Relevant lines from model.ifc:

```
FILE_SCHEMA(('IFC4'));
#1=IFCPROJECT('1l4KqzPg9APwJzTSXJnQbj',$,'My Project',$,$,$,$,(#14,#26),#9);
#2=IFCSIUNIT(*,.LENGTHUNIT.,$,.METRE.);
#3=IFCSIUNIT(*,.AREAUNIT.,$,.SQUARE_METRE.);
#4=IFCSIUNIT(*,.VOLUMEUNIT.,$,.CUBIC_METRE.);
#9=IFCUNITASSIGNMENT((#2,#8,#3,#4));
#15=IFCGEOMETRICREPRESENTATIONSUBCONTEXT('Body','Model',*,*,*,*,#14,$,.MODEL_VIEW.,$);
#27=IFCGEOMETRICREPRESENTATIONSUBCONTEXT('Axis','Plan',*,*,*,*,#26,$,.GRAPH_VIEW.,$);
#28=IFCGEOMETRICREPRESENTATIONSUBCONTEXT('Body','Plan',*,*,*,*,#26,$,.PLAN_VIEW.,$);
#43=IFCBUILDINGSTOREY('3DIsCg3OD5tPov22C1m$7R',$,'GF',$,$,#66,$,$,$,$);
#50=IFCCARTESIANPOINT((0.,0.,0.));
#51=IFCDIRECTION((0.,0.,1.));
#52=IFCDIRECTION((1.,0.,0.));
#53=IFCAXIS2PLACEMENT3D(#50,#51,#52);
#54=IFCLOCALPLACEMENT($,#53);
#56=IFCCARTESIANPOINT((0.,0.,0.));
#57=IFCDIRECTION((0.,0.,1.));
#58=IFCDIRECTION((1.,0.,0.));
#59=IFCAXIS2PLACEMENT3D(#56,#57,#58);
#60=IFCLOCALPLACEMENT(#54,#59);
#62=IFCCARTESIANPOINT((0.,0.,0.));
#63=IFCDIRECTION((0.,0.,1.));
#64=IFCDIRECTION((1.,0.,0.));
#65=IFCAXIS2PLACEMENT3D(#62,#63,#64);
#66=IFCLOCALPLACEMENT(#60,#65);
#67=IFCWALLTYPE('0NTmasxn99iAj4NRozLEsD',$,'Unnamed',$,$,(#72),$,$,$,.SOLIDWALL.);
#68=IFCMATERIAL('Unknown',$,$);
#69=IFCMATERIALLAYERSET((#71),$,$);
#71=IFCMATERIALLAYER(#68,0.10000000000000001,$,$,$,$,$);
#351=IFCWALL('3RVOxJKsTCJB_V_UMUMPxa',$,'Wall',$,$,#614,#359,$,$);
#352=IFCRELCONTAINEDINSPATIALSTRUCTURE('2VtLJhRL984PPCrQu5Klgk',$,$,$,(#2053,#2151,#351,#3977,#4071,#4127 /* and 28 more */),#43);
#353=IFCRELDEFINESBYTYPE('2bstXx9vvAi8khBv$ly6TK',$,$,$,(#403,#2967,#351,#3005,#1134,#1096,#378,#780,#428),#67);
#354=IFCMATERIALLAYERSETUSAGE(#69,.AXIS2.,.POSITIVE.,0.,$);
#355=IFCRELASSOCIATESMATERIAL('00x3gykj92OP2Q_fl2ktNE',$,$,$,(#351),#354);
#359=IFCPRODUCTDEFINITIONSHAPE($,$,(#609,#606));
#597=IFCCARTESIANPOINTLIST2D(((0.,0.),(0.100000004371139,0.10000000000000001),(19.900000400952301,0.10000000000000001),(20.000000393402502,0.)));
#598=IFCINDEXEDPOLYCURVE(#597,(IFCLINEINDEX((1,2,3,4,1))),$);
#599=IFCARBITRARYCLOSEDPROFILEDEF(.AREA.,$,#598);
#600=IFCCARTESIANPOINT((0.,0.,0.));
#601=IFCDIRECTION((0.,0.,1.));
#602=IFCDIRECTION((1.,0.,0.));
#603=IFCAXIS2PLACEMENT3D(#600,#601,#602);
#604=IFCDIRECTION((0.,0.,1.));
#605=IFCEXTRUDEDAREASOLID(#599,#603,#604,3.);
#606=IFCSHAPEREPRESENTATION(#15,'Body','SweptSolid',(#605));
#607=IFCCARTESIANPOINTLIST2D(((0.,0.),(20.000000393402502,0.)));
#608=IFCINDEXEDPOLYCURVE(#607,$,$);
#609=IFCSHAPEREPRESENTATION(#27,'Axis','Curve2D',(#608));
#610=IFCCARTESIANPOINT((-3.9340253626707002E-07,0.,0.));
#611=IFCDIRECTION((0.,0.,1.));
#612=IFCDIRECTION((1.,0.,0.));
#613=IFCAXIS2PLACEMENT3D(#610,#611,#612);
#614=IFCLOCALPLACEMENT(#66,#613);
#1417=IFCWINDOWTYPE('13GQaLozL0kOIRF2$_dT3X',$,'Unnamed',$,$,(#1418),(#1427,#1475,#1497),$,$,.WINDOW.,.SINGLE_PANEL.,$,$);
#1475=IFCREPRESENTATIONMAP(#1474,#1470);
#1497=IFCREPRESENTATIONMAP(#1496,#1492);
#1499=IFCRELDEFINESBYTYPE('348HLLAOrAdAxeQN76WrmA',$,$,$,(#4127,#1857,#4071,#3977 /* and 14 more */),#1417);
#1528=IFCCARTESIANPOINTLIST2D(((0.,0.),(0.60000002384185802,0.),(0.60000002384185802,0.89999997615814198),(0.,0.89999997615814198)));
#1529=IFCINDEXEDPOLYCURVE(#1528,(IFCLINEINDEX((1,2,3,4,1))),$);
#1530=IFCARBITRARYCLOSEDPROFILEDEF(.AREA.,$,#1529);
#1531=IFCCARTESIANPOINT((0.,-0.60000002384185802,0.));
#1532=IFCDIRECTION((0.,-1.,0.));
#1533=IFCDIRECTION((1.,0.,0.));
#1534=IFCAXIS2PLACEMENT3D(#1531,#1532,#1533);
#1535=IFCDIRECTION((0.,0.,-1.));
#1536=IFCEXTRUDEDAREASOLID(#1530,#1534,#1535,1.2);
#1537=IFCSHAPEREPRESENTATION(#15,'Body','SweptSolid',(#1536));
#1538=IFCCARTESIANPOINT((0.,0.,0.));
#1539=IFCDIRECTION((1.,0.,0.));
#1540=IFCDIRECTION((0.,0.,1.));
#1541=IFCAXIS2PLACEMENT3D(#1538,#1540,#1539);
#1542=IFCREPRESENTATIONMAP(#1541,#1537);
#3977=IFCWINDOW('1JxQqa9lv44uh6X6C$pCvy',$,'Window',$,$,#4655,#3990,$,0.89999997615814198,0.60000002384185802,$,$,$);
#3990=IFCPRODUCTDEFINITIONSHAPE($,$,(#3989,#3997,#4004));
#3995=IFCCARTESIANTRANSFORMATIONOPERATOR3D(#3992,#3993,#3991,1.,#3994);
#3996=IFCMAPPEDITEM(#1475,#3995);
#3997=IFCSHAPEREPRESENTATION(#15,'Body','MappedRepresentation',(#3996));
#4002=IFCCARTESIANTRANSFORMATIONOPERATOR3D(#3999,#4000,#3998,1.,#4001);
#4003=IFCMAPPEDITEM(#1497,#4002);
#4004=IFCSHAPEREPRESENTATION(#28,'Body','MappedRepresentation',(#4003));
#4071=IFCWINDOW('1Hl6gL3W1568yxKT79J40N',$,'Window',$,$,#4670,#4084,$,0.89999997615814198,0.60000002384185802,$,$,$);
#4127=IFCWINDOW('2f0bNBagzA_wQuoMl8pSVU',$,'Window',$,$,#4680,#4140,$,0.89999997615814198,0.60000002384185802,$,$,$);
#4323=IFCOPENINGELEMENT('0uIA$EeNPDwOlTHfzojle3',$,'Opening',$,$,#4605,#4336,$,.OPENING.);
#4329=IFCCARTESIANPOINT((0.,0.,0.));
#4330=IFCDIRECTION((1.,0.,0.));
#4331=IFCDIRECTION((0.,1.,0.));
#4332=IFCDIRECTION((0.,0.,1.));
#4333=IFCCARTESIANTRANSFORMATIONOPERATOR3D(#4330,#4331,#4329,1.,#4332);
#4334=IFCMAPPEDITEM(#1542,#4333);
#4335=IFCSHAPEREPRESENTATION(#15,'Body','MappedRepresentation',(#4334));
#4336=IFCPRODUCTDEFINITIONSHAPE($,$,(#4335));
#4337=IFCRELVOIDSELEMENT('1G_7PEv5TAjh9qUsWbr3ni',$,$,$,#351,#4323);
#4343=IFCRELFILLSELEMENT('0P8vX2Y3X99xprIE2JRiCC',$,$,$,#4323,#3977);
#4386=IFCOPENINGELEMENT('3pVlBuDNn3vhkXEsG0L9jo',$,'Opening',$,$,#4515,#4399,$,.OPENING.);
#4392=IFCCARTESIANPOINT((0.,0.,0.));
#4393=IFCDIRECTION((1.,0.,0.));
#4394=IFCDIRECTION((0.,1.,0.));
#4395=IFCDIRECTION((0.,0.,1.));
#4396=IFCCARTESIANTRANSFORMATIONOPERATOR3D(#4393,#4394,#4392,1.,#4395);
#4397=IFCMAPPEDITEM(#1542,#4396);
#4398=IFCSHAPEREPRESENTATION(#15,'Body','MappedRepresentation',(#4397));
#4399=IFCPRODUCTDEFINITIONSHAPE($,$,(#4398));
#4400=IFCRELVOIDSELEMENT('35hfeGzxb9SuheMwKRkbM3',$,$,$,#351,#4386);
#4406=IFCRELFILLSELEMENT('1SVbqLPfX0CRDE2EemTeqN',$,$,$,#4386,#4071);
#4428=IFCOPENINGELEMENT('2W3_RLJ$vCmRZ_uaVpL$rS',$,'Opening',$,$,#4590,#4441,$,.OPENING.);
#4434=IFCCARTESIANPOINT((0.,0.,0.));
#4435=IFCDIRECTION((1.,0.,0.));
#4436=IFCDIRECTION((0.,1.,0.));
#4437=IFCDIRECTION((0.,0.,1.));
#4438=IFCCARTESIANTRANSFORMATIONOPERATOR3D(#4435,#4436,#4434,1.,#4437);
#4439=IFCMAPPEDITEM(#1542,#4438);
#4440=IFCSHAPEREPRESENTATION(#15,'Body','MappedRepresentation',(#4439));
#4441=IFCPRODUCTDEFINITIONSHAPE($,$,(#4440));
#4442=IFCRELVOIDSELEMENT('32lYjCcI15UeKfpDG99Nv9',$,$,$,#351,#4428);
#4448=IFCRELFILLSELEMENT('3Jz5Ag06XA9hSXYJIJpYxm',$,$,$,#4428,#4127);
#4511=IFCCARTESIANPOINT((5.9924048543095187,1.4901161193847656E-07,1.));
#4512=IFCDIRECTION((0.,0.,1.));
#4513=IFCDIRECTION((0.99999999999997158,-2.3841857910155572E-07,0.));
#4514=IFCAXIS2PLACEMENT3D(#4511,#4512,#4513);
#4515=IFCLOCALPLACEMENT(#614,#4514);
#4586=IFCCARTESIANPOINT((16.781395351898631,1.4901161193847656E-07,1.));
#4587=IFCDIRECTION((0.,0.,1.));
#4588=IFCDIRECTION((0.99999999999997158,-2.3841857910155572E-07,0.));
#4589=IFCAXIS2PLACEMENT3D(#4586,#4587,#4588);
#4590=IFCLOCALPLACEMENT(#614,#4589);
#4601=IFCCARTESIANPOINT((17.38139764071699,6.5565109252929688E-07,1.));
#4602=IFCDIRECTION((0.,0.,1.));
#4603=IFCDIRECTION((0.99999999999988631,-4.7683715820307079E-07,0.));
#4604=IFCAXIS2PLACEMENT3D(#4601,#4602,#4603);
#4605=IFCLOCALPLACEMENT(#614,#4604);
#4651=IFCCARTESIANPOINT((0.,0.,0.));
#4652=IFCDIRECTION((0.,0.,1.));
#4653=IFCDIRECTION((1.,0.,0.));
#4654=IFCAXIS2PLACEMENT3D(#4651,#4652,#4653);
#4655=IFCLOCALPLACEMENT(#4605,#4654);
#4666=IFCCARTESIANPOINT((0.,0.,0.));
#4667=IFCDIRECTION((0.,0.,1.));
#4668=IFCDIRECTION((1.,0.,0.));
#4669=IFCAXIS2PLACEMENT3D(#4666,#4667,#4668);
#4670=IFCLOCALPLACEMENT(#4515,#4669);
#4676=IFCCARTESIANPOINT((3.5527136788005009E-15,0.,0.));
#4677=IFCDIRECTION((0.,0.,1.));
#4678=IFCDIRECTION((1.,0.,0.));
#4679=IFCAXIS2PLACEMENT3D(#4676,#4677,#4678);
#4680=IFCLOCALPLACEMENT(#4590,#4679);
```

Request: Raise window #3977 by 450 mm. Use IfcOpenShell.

```python
import numpy as np
import ifcopenshell
import ifcopenshell.api.geometry
import ifcopenshell.util.placement
import ifcopenshell.util.unit

model = ifcopenshell.open("model.ifc")
unit_scale = ifcopenshell.util.unit.calculate_unit_scale(model)

window = model.by_guid("1JxQqa9lv44uh6X6C$pCvy")
opening = window.FillsVoids[0].RelatingOpeningElement
dz = 0.45

shift = np.array([0.0, 0.0, dz])
# The window is placed relative to its opening, so it follows when the opening moves.
matrix = ifcopenshell.util.placement.get_local_placement(opening.ObjectPlacement)
matrix[:3, 3] += shift
ifcopenshell.api.geometry.edit_object_placement(
    model, product=opening, matrix=matrix, is_si=False, should_transform_children=True
)

print(f"moved by {dz * unit_scale:+.3f} m")

model.write("model_updated.ifc")
```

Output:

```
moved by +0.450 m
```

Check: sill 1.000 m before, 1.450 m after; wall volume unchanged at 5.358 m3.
